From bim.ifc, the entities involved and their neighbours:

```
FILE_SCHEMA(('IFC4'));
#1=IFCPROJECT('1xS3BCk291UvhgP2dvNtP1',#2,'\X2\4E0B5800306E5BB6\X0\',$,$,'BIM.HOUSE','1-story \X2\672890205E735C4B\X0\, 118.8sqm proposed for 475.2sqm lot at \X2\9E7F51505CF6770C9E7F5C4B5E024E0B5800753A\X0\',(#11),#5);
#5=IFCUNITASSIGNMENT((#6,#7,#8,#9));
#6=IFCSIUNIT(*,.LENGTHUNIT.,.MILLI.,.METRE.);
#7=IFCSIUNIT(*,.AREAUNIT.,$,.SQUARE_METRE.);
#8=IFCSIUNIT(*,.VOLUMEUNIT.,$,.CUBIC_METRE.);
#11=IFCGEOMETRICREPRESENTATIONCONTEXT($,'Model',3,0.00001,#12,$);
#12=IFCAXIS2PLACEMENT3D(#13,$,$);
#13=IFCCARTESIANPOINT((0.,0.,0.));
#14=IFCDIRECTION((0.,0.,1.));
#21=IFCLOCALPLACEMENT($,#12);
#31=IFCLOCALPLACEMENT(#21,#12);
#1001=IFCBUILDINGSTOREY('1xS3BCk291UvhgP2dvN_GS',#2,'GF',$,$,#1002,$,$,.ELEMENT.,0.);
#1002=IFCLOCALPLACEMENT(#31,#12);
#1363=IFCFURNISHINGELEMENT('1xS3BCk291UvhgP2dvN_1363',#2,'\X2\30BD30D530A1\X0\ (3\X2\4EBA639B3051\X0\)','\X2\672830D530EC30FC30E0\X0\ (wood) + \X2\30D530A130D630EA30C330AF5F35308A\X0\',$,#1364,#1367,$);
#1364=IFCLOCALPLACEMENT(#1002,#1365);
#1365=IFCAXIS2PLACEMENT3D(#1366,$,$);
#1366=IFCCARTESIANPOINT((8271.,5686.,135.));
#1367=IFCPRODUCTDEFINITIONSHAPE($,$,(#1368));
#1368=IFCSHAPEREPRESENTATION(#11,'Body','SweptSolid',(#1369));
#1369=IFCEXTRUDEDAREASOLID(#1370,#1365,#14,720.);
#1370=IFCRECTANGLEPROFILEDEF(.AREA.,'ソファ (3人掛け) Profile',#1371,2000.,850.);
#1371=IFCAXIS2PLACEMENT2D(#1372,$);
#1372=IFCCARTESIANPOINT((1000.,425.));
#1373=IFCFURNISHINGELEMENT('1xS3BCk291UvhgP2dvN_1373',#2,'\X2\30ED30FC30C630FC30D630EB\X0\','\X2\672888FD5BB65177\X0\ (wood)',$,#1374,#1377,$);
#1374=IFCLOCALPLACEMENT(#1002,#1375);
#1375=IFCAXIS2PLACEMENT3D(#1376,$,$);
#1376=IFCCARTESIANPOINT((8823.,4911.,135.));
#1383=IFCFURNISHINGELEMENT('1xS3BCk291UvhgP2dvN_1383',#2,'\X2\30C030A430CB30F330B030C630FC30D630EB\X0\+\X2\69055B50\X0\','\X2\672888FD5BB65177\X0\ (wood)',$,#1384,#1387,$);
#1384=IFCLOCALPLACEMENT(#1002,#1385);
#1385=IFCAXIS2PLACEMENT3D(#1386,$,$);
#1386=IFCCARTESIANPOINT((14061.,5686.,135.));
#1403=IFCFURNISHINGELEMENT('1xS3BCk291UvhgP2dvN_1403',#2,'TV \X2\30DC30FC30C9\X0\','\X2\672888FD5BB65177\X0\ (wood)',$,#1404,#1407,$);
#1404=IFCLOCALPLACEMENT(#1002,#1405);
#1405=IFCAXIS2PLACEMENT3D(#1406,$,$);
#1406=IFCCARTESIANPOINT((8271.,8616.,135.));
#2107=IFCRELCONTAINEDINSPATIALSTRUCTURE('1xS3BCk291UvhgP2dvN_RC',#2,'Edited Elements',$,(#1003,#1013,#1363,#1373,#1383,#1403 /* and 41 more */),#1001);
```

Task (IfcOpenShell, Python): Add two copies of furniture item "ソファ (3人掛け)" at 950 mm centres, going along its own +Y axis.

```python
import ifcopenshell
import ifcopenshell.api.geometry
import ifcopenshell.api.root
import ifcopenshell.util.element
import ifcopenshell.util.placement

model = ifcopenshell.open("bim.ifc")


def reuse_history(source, copy):
    """copy_class also copies each property set's owner history, people and application; keep the originals."""
    for rel in copy.IsDefinedBy:
        if rel.is_a("IfcRelDefinesByProperties") and (history := rel.RelatingPropertyDefinition.OwnerHistory):
            rel.RelatingPropertyDefinition.OwnerHistory = source.OwnerHistory
            ifcopenshell.util.element.remove_deep2(model, history)


source = model.by_id(1363)
base = ifcopenshell.util.placement.get_local_placement(source.ObjectPlacement)
step = base[:3, 1] * 950.0

for i in range(1, 3):
    copy = ifcopenshell.api.root.copy_class(model, product=source)
    copy.Representation = ifcopenshell.util.element.copy_deep(
        model, source.Representation, exclude=["IfcGeometricRepresentationContext", "IfcRepresentationMap"]
    )
    reuse_history(source, copy)
    matrix = base.copy()
    matrix[:3, 3] += i * step
    print("added at", matrix[:3, 3].round(3) + 0.0)
    ifcopenshell.api.geometry.edit_object_placement(model, product=copy, matrix=matrix, is_si=False)

model.write("bim_rev.ifc")
```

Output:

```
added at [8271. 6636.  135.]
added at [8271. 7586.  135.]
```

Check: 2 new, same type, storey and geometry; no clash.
